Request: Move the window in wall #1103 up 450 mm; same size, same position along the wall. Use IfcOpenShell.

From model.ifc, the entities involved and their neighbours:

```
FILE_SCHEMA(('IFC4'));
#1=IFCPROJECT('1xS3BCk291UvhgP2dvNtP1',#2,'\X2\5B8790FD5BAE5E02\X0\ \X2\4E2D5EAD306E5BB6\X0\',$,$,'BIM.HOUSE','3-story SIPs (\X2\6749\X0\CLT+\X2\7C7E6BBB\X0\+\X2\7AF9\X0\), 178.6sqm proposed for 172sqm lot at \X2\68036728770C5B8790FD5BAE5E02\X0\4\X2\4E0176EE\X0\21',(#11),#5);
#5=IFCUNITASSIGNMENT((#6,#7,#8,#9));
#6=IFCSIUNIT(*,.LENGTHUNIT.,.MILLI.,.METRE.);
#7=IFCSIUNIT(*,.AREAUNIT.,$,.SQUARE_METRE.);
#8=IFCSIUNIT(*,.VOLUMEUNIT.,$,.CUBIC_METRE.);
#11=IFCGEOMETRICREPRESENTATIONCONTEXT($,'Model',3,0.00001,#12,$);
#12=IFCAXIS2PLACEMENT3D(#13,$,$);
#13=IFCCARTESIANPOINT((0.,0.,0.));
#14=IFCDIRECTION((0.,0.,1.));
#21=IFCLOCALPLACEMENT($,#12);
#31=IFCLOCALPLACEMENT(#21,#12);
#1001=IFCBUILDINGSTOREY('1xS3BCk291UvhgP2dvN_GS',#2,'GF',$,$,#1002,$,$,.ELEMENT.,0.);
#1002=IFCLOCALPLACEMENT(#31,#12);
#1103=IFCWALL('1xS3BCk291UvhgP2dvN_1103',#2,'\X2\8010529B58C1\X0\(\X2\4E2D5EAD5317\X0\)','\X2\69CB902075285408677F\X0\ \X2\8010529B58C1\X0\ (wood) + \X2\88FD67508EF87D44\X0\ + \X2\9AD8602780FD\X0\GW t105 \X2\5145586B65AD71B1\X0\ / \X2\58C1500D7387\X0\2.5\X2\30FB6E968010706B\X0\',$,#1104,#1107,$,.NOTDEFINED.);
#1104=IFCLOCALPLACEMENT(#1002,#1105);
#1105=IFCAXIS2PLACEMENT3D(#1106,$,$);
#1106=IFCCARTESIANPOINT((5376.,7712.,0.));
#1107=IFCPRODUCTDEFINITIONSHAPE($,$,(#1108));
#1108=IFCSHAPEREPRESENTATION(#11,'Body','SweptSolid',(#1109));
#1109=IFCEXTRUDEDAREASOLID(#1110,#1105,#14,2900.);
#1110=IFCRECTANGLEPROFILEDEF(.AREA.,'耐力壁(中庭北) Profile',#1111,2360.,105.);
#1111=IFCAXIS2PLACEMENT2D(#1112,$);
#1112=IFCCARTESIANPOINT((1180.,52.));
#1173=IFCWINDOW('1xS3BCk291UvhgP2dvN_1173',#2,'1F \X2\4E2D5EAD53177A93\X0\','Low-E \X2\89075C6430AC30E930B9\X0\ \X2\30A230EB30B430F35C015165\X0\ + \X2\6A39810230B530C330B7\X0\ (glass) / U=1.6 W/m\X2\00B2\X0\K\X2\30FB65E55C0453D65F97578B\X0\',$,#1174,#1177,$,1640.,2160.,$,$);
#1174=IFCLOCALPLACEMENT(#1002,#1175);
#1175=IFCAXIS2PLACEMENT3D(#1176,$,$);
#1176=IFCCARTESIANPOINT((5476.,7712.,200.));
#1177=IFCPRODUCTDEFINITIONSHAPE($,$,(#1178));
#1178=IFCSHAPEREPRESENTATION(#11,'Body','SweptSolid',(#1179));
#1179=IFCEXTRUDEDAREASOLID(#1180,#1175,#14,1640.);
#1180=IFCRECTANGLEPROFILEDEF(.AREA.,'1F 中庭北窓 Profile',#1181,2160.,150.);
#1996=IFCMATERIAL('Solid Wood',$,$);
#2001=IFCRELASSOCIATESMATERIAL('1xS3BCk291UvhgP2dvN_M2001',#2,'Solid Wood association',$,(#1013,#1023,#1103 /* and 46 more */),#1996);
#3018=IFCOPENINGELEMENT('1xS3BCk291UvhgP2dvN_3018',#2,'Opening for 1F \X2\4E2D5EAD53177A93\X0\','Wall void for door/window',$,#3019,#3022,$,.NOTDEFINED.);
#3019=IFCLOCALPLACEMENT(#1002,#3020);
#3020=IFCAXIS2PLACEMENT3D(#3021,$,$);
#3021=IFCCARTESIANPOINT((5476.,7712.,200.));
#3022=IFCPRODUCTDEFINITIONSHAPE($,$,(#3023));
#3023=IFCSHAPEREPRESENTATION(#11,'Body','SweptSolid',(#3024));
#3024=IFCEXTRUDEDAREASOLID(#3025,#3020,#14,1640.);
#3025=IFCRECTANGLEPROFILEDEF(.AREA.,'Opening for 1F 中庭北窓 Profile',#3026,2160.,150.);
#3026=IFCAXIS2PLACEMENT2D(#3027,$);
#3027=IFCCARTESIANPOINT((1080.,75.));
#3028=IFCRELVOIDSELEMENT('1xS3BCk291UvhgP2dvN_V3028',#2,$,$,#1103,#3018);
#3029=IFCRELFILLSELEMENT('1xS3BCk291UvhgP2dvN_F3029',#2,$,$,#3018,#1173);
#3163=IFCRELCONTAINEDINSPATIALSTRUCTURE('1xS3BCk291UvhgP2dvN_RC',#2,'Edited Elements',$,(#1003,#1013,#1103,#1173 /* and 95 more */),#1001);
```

```python
import numpy as np
import ifcopenshell
import ifcopenshell.api.geometry
import ifcopenshell.util.placement
import ifcopenshell.util.unit

model = ifcopenshell.open("model.ifc")
unit_scale = ifcopenshell.util.unit.calculate_unit_scale(model)

window = model.by_guid("1xS3BCk291UvhgP2dvN_1173")
opening = window.FillsVoids[0].RelatingOpeningElement
dz = 0.45 / unit_scale

shift = np.array([0.0, 0.0, dz])
# The window is not placed relative to its opening, so move both.
for product in (opening, window):
    matrix = ifcopenshell.util.placement.get_local_placement(product.ObjectPlacement)
    matrix[:3, 3] += shift
    ifcopenshell.api.geometry.edit_object_placement(model, product=product, matrix=matrix, is_si=False)

print(f"moved by {dz * unit_scale:+.3f} m")

model.write("model-out.ifc")
```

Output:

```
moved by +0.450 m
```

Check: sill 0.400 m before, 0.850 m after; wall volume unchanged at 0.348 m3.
